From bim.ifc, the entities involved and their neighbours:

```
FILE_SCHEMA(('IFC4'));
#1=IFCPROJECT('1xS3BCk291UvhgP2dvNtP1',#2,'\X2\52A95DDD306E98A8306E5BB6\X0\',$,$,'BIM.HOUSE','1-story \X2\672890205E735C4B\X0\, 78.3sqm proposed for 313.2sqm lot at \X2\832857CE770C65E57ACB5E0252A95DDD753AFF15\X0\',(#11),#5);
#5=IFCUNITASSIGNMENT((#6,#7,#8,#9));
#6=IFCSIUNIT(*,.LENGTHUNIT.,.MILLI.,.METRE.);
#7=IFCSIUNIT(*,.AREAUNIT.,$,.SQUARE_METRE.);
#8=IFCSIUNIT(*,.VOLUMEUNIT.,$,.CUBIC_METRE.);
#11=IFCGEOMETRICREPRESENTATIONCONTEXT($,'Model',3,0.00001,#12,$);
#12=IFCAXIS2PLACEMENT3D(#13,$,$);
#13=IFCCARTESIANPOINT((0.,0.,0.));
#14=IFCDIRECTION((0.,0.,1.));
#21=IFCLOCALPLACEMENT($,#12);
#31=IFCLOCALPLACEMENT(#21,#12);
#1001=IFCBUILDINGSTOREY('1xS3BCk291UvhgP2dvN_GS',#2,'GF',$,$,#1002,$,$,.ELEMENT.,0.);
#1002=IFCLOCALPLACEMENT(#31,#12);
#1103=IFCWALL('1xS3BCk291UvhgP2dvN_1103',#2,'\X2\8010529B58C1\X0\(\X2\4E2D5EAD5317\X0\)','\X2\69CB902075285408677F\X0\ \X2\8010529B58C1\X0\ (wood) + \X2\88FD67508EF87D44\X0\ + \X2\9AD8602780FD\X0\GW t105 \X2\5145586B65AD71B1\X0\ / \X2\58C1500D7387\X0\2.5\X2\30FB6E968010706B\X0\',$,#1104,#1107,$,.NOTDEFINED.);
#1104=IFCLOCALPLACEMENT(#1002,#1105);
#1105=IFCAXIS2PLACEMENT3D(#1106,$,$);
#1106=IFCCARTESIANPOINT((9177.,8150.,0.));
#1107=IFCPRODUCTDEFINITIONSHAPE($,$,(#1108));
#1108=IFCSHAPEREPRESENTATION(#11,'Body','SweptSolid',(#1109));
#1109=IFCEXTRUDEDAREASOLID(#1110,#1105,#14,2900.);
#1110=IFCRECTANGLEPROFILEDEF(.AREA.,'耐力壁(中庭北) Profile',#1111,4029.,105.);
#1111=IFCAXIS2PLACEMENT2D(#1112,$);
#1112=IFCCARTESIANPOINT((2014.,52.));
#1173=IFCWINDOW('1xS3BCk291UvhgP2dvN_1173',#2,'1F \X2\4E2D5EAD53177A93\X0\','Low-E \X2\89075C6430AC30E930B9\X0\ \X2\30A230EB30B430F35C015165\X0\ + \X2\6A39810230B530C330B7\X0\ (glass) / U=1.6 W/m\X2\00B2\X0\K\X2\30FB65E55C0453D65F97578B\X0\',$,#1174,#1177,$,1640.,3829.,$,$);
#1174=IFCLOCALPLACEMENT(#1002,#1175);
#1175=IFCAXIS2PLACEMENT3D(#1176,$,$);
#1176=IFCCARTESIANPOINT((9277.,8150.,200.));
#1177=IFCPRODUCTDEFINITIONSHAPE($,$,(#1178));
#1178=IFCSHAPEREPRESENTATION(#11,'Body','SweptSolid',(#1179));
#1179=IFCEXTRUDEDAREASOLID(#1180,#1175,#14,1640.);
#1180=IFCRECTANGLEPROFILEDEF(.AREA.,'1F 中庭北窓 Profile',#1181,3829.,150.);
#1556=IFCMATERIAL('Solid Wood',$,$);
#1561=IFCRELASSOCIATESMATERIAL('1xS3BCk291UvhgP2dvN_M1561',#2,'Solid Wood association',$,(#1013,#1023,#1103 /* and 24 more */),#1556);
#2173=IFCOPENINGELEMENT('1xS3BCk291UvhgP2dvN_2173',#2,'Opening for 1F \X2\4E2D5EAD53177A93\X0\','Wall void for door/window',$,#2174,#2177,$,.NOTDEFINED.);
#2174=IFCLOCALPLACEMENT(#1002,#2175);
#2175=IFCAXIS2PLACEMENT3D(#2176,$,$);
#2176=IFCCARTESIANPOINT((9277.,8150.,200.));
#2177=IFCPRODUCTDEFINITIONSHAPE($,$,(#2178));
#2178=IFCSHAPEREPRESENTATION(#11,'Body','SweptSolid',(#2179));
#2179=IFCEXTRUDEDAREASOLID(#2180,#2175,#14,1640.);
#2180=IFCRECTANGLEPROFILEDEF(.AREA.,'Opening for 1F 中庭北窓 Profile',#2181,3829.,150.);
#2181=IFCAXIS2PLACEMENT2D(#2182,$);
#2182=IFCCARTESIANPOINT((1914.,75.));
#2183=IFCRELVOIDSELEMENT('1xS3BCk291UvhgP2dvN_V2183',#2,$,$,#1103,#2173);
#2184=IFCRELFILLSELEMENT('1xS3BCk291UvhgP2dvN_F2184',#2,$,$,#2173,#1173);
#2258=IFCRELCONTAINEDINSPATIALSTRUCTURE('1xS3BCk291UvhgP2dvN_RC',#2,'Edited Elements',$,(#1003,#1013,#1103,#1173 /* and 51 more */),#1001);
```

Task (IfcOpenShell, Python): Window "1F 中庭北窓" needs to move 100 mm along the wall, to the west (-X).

```python
import ifcopenshell
import ifcopenshell.api.geometry
import ifcopenshell.util.placement

model = ifcopenshell.open("bim.ifc")

window = model.by_guid("1xS3BCk291UvhgP2dvN_1173")
opening = window.FillsVoids[0].RelatingOpeningElement
wall = opening.VoidsElements[0].RelatingBuildingElement

wall_matrix = ifcopenshell.util.placement.get_local_placement(wall.ObjectPlacement)
shift = wall_matrix[:3, 0] * -100.0
before = ifcopenshell.util.placement.get_local_placement(window.ObjectPlacement)[:3, 3].copy()

# The window is not placed relative to its opening, so move both.
for product in (opening, window):
    matrix = ifcopenshell.util.placement.get_local_placement(product.ObjectPlacement)
    matrix[:3, 3] += shift
    ifcopenshell.api.geometry.edit_object_placement(model, product=product, matrix=matrix, is_si=False)

after = ifcopenshell.util.placement.get_local_placement(window.ObjectPlacement)[:3, 3]
print("window moved by", (after - before).round(3) + 0.0)

model.write("bim_v2.ifc")
```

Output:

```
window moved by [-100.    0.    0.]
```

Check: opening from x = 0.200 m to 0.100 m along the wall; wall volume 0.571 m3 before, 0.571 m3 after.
